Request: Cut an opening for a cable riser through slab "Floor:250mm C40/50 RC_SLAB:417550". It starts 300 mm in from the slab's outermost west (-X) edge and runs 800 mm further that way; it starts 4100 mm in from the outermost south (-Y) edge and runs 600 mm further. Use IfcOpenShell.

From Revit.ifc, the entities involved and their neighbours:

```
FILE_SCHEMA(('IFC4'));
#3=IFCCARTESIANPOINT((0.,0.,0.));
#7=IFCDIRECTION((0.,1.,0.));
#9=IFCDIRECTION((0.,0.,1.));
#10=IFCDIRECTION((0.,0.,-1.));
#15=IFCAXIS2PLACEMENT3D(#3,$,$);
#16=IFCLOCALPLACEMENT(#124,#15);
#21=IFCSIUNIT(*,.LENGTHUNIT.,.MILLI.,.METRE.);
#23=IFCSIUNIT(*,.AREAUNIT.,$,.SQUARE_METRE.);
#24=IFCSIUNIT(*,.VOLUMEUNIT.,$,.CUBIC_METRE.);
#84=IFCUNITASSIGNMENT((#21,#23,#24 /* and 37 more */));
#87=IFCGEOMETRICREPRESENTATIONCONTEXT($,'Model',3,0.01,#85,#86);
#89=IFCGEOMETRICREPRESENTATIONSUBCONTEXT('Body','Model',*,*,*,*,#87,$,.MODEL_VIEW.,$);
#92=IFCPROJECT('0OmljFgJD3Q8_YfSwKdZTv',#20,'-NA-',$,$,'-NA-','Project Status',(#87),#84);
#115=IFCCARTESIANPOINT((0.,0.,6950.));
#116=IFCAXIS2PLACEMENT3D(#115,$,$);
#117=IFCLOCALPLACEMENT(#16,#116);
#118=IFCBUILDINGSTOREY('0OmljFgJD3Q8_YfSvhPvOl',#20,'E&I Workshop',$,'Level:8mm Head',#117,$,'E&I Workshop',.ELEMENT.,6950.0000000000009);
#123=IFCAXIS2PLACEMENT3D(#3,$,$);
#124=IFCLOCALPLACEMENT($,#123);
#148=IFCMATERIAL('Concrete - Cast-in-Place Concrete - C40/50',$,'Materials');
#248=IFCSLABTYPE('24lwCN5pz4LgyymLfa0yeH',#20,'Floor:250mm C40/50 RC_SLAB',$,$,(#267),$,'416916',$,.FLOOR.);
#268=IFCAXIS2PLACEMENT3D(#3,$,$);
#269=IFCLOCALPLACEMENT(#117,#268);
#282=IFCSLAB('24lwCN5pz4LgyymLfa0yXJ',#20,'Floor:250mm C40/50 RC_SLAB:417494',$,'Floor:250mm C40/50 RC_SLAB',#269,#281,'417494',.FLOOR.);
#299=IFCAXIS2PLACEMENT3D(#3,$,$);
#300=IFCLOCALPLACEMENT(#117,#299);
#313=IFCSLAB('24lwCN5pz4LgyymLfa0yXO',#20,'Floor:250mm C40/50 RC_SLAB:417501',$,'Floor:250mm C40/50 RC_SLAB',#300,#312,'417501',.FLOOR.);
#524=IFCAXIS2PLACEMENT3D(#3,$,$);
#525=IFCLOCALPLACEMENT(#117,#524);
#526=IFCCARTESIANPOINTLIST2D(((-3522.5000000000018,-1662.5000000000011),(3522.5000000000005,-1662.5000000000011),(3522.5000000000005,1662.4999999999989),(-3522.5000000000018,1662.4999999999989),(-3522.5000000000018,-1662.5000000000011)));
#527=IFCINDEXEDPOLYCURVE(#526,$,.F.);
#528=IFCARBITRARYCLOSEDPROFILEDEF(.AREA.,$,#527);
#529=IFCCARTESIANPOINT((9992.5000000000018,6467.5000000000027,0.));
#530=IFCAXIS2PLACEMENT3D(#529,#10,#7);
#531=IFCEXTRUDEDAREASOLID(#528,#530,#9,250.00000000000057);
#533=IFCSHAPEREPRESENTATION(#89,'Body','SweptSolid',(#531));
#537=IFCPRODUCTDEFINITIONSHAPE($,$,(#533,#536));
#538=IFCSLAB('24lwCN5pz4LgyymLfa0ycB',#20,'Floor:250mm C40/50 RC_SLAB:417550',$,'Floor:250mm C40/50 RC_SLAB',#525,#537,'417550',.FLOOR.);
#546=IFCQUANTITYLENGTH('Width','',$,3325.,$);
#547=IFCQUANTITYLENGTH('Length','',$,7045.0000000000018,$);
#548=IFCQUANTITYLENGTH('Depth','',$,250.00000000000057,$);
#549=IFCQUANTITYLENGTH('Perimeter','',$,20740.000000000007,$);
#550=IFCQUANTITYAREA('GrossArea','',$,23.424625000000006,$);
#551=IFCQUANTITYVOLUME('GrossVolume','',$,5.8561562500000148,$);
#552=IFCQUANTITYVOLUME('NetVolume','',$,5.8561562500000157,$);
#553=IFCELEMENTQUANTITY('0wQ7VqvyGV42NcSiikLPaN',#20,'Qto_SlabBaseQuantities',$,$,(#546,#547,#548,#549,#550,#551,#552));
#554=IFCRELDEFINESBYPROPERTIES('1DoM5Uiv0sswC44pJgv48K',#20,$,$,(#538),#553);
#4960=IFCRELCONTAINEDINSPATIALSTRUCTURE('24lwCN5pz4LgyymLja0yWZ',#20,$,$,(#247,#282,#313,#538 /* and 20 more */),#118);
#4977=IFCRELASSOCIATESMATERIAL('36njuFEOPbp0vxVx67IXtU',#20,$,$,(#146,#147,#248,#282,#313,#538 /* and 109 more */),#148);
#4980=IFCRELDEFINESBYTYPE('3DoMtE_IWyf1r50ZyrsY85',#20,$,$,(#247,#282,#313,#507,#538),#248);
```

```python
import numpy as np
import ifcopenshell
import ifcopenshell.api.feature
import ifcopenshell.api.geometry
import ifcopenshell.api.pset
import ifcopenshell.api.root
import ifcopenshell.geom
import ifcopenshell.util.element
import ifcopenshell.util.placement
import ifcopenshell.util.representation
import ifcopenshell.util.shape
import ifcopenshell.util.unit

model = ifcopenshell.open("Revit.ifc")
unit_scale = ifcopenshell.util.unit.calculate_unit_scale(model)
volume_scale = ifcopenshell.util.unit.calculate_unit_scale(model, "VOLUMEUNIT")
settings = ifcopenshell.geom.settings()


def volume(element):
    """Net volume in cubic metres, openings subtracted."""
    shape = ifcopenshell.geom.create_shape(settings, element)
    return ifcopenshell.util.shape.get_volume(shape.geometry)


slab = model.by_id(538)
before = volume(slab)

# Extent in the slab's own axes, in metres. The edges named are its -X and -Y sides.
slab_shape = ifcopenshell.geom.create_shape(settings, slab)
vertices = ifcopenshell.util.shape.get_vertices(slab_shape.geometry)
x_min, y_min, bottom = vertices.min(axis=0)
top = vertices[:, 2].max()

opening = ifcopenshell.api.root.create_entity(model, ifc_class="IfcOpeningElement", name="Cable riser opening", predefined_type="OPENING")
context = ifcopenshell.util.representation.get_context(model, "Model", "Body", "MODEL_VIEW")
width, depth = 0.8, 0.6
outline = [(0.0, 0.0), (width, 0.0), (width, depth), (0.0, depth), (0.0, 0.0)]
# Overshoot both faces by 50 mm so the cut is clean.
shape = ifcopenshell.api.geometry.add_slab_representation(
    model, context=context, depth=top - bottom + 0.1, polyline=outline
)
ifcopenshell.api.geometry.assign_representation(model, product=opening, representation=shape)

matrix = ifcopenshell.util.placement.get_local_placement(slab.ObjectPlacement)
matrix[:, 3] = matrix @ np.append(np.array([x_min + 0.3, y_min + 4.1, bottom - 0.05]) / unit_scale, 1.0)
ifcopenshell.api.geometry.edit_object_placement(model, product=opening, matrix=matrix, is_si=False)
ifcopenshell.api.feature.add_feature(model, feature=opening, element=slab)

after = volume(slab)

# Update the slab's stored quantities.
qto = model.by_id(ifcopenshell.util.element.get_pset(slab, "Qto_SlabBaseQuantities", should_inherit=False)["id"])
ifcopenshell.api.pset.edit_qto(model, qto=qto, properties={"NetVolume": after / volume_scale})

print(f"slab volume {before:.3f} -> {after:.3f} m3")

model.write("Revit_v2.ifc")
```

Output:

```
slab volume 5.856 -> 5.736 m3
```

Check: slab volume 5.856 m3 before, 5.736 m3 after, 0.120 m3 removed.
